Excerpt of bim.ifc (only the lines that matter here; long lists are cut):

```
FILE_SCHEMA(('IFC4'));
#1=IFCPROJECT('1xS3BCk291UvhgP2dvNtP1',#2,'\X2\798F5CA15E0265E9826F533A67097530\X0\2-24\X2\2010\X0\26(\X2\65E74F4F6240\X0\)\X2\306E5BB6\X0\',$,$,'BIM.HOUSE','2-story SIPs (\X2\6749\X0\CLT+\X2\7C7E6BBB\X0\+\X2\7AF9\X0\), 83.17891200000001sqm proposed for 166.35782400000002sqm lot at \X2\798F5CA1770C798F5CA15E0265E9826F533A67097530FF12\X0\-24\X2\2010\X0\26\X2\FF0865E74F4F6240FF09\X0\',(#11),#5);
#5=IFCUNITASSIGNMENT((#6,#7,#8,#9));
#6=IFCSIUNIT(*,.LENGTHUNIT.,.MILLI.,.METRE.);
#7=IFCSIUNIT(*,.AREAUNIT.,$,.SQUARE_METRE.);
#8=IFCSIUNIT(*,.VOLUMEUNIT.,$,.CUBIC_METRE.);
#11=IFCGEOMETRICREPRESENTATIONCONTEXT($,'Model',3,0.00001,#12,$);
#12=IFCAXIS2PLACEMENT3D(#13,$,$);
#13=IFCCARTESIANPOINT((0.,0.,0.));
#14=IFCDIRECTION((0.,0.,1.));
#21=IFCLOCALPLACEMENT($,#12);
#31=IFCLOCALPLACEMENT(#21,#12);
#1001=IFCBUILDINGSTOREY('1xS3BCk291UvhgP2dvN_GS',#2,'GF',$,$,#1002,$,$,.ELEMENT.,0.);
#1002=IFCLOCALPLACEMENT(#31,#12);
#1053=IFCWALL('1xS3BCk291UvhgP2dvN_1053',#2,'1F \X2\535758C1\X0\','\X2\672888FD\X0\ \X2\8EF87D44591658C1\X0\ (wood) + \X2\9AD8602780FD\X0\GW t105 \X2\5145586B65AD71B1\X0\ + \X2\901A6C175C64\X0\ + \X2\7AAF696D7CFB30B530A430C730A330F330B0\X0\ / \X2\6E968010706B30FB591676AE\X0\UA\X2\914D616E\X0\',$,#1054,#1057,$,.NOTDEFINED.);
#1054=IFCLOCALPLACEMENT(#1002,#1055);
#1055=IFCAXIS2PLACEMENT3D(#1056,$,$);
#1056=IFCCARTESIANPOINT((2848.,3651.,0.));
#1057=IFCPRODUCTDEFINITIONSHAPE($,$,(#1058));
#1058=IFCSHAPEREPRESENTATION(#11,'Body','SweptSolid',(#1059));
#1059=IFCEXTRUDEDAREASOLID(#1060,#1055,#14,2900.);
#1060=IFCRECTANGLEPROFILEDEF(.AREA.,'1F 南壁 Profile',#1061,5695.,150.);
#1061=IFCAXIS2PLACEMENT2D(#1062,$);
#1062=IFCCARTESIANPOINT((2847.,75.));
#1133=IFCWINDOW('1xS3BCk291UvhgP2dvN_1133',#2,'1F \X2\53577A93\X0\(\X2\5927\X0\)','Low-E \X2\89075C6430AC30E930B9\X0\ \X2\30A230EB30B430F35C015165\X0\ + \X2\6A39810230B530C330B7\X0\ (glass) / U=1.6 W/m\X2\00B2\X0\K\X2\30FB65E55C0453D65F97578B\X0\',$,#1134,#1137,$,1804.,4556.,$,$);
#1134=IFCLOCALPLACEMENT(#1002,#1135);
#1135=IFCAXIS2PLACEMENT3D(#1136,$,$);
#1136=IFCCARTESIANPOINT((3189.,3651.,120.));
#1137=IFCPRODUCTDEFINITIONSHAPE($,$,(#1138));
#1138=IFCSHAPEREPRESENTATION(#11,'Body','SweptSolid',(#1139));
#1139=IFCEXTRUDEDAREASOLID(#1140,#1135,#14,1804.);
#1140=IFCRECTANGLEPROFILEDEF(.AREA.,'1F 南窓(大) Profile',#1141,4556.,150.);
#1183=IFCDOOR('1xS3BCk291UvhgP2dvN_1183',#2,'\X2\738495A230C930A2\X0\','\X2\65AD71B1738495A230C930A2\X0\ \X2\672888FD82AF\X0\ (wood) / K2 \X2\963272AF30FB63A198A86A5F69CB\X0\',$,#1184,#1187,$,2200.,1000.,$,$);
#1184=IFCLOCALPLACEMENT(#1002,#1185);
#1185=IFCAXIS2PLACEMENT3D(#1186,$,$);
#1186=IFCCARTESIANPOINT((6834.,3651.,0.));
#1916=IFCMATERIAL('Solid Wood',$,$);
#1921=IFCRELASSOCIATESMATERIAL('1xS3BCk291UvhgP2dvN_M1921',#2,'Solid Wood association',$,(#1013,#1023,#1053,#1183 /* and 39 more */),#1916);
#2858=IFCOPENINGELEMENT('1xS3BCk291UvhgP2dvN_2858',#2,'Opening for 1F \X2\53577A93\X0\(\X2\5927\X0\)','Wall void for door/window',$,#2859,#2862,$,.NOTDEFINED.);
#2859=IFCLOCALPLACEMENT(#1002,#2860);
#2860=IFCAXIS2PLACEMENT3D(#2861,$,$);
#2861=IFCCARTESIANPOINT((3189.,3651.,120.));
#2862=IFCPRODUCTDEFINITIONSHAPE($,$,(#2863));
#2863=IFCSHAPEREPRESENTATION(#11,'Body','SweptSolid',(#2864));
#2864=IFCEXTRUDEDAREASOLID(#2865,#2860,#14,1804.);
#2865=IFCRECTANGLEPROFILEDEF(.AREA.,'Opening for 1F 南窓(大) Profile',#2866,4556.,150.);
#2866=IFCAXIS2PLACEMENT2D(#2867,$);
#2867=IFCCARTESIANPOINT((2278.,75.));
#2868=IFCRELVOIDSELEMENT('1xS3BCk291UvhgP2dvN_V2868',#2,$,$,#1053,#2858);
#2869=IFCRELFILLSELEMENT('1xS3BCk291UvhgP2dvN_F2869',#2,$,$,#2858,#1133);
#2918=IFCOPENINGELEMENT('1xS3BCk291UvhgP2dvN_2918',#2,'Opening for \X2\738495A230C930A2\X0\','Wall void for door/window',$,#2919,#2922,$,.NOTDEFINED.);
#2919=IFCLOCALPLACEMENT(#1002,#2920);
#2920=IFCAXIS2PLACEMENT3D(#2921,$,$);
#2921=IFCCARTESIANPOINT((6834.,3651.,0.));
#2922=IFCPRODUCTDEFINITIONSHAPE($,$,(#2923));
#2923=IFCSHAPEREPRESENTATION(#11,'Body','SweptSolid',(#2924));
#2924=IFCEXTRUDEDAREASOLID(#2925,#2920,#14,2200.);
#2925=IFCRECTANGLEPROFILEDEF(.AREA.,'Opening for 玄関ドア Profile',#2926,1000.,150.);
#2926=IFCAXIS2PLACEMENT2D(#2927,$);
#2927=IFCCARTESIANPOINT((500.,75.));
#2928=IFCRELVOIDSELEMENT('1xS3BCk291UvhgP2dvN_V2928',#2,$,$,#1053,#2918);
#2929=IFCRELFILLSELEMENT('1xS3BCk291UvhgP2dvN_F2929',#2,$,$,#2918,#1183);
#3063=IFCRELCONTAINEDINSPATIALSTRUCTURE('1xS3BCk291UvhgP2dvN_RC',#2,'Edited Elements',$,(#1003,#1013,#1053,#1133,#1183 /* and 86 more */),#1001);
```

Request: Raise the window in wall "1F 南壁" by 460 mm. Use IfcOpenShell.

```python
import numpy as np
import ifcopenshell
import ifcopenshell.api.geometry
import ifcopenshell.util.placement
import ifcopenshell.util.unit

model = ifcopenshell.open("bim.ifc")
unit_scale = ifcopenshell.util.unit.calculate_unit_scale(model)

window = model.by_guid("1xS3BCk291UvhgP2dvN_1133")
opening = window.FillsVoids[0].RelatingOpeningElement
dz = 0.46 / unit_scale

shift = np.array([0.0, 0.0, dz])
# The window is not placed relative to its opening, so move both.
for product in (opening, window):
    matrix = ifcopenshell.util.placement.get_local_placement(product.ObjectPlacement)
    matrix[:3, 3] += shift
    ifcopenshell.api.geometry.edit_object_placement(model, product=product, matrix=matrix, is_si=False)

print(f"moved by {dz * unit_scale:+.3f} m")

model.write("bim-out.ifc")
```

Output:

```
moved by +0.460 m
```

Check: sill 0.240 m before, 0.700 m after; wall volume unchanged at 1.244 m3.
